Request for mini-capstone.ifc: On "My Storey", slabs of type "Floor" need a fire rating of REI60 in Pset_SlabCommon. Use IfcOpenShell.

First a look at what the model holds.

```python
import ifcopenshell
import ifcopenshell.util.element

model = ifcopenshell.open("mini-capstone.ifc")
print(model.schema)
storey = next(s for s in model.by_type("IfcBuildingStorey") if s.Name == "My Storey")
slabs = [e for e in ifcopenshell.util.element.get_decomposition(storey) if e.is_a("IfcSlab")]
seen = {}
for e in slabs:
    element_type = ifcopenshell.util.element.get_type(e)
    key = (element_type.Name if element_type != e and element_type else None, ifcopenshell.util.element.get_pset(e, "Pset_SlabCommon", "FireRating"))
    seen[key] = seen.get(key, 0) + 1
for (name, value), count in sorted(seen.items(), key=str):
    print(count, "x", name, "|", value)
```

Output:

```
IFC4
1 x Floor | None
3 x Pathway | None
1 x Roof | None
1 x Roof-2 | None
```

```python
import ifcopenshell
import ifcopenshell.api.pset
import ifcopenshell.util.element

model = ifcopenshell.open("mini-capstone.ifc")

storey = next(s for s in model.by_type("IfcBuildingStorey") if s.Name == "My Storey")
slabs = [e for e in ifcopenshell.util.element.get_decomposition(storey) if e.is_a("IfcSlab")]

count = 0
for e in slabs:
    element_type = ifcopenshell.util.element.get_type(e)
    if element_type in (None, e) or element_type.Name != "Floor":
        continue
    # add_pset returns the element's existing set when there is one.
    pset = ifcopenshell.api.pset.add_pset(model, product=e, name="Pset_SlabCommon")
    ifcopenshell.api.pset.edit_pset(model, pset=pset, properties={"FireRating": "REI60"})
    count += 1

print(count, "slabs updated")

model.write("mini-capstone_edited.ifc")
```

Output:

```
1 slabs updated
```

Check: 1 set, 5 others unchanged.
